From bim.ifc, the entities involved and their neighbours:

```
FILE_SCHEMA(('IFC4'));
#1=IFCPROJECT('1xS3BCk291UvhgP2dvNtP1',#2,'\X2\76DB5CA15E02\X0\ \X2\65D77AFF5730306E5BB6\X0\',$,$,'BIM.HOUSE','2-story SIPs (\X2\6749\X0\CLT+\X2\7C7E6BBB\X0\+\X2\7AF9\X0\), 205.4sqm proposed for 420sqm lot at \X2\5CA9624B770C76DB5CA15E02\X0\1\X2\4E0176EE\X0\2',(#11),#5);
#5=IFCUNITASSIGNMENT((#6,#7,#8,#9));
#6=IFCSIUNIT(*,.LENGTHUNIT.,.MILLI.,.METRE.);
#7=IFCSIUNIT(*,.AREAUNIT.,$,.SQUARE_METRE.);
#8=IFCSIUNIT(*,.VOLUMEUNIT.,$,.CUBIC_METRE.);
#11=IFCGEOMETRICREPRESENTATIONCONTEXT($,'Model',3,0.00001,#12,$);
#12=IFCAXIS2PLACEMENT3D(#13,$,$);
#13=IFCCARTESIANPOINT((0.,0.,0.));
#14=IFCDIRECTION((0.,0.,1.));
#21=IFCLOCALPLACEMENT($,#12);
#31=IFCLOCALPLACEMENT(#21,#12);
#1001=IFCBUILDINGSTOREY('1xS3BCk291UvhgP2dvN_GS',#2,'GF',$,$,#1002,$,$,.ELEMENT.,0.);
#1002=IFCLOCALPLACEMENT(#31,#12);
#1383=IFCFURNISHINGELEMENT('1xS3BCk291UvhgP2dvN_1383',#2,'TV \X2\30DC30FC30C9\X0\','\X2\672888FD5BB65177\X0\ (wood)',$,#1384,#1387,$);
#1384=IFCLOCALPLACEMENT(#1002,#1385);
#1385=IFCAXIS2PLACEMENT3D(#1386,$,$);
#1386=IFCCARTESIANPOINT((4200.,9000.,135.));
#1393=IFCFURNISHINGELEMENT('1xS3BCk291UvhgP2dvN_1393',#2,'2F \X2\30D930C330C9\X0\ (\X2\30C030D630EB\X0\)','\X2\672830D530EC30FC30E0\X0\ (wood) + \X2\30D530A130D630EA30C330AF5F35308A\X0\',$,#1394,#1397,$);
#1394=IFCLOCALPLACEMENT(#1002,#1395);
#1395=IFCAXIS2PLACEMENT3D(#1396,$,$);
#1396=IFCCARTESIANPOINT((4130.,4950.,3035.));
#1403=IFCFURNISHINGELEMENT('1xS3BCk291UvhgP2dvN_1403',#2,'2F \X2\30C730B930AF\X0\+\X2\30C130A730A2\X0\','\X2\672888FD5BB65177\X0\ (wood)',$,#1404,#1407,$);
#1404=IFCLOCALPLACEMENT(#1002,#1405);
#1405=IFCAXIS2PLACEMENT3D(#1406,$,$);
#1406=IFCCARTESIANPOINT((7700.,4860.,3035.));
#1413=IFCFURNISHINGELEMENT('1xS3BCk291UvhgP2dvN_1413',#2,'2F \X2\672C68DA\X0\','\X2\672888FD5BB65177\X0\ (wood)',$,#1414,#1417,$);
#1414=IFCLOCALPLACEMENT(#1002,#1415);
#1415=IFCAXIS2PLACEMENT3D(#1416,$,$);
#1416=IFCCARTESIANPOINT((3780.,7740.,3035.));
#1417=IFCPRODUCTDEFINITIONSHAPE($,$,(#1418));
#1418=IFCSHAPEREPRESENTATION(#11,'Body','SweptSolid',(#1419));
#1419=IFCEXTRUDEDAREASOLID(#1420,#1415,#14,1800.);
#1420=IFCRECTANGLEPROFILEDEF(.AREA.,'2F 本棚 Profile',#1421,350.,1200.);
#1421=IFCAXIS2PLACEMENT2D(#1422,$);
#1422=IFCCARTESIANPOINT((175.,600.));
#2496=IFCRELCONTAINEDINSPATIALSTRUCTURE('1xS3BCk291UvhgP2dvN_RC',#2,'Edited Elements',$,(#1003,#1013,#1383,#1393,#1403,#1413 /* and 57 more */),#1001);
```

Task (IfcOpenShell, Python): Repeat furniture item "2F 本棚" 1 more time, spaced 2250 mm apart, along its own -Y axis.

```python
import ifcopenshell
import ifcopenshell.api.geometry
import ifcopenshell.api.root
import ifcopenshell.util.element
import ifcopenshell.util.placement
import ifcopenshell.util.unit

model = ifcopenshell.open("bim.ifc")
unit_scale = ifcopenshell.util.unit.calculate_unit_scale(model)


def reuse_history(source, copy):
    """copy_class also copies each property set's owner history, people and application; keep the originals."""
    for rel in copy.IsDefinedBy:
        if rel.is_a("IfcRelDefinesByProperties") and (history := rel.RelatingPropertyDefinition.OwnerHistory):
            rel.RelatingPropertyDefinition.OwnerHistory = source.OwnerHistory
            ifcopenshell.util.element.remove_deep2(model, history)


source = model.by_id(1413)
base = ifcopenshell.util.placement.get_local_placement(source.ObjectPlacement)
step = -base[:3, 1] * 2.25 / unit_scale

for i in range(1, 2):
    copy = ifcopenshell.api.root.copy_class(model, product=source)
    copy.Representation = ifcopenshell.util.element.copy_deep(
        model, source.Representation, exclude=["IfcGeometricRepresentationContext", "IfcRepresentationMap"]
    )
    reuse_history(source, copy)
    matrix = base.copy()
    matrix[:3, 3] += i * step
    print("added at", matrix[:3, 3].round(3) + 0.0)
    ifcopenshell.api.geometry.edit_object_placement(model, product=copy, matrix=matrix, is_si=False)

model.write("bim-out.ifc")
```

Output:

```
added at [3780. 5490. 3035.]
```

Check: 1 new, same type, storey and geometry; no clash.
